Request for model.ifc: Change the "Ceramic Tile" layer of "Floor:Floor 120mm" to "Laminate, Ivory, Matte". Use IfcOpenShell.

First a look at what the model holds.

```python
import ifcopenshell
import ifcopenshell.util.element

model = ifcopenshell.open("model.ifc")
print(model.schema)
for layer_set in model.by_type("IfcMaterialLayerSet"):
    if layer_set.LayerSetName == "Floor:Floor 120mm":
        for layer in layer_set.MaterialLayers:
            print(layer.id(), layer.Material and layer.Material.Name, layer.LayerThickness, sep=" | ")
        print(len(ifcopenshell.util.element.get_elements_by_material(model, layer_set)), "elements and types use it")
print(sorted(m.Name for m in model.by_type("IfcMaterial") if m.Name)[:60])
```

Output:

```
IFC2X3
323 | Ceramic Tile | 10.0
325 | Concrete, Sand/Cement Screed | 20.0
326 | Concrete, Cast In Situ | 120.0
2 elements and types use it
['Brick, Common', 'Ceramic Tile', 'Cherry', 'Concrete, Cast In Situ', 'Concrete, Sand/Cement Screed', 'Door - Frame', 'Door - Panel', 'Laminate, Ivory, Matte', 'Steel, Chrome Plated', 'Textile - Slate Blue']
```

```python
import ifcopenshell
import ifcopenshell.api.material

model = ifcopenshell.open("model.ifc")

layer_set = next(s for s in model.by_type("IfcMaterialLayerSet") if s.LayerSetName == "Floor:Floor 120mm")
layer = next(l for l in layer_set.MaterialLayers if l.Material and l.Material.Name == "Ceramic Tile")
material = next(m for m in model.by_type("IfcMaterial") if m.Name == "Laminate, Ivory, Matte")

# Point this one layer at the other material; renaming the old one would change it everywhere.
ifcopenshell.api.material.edit_layer(model, layer=layer, attributes={}, material=material)

print([l.Material.Name if l.Material else None for l in layer_set.MaterialLayers])

model.write("model_updated.ifc")
```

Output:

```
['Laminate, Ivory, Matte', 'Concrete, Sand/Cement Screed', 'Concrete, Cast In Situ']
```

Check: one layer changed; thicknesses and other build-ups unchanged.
